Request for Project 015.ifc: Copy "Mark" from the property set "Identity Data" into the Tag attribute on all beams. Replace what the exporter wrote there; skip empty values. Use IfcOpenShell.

First a look at what the model holds.

```python
import ifcopenshell
import ifcopenshell.util.element

model = ifcopenshell.open("Project 015.ifc")
print(model.schema)
beams = model.by_type("IfcBeam")
print(len(beams), "beams")
for e in beams[:8]:
    source = ifcopenshell.util.element.get_pset(e, "Identity Data", "Mark")
    target = e.Tag
    print(e.id(), repr(source), repr(target), sep=" | ")
```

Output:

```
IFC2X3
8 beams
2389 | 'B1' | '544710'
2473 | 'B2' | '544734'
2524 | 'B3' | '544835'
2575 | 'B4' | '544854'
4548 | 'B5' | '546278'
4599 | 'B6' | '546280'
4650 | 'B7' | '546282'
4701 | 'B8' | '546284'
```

```python
import ifcopenshell
import ifcopenshell.util.element

model = ifcopenshell.open("Project 015.ifc")

count = 0
for e in model.by_type("IfcBeam"):
    value = ifcopenshell.util.element.get_pset(e, "Identity Data", "Mark")
    current = e.Tag
    if not value or not value.strip() or current == value:
        continue
    e.Tag = value
    count += 1

print(count, "beams updated")

model.write("Project 015_v2.ifc")
```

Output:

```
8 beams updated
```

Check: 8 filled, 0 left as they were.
